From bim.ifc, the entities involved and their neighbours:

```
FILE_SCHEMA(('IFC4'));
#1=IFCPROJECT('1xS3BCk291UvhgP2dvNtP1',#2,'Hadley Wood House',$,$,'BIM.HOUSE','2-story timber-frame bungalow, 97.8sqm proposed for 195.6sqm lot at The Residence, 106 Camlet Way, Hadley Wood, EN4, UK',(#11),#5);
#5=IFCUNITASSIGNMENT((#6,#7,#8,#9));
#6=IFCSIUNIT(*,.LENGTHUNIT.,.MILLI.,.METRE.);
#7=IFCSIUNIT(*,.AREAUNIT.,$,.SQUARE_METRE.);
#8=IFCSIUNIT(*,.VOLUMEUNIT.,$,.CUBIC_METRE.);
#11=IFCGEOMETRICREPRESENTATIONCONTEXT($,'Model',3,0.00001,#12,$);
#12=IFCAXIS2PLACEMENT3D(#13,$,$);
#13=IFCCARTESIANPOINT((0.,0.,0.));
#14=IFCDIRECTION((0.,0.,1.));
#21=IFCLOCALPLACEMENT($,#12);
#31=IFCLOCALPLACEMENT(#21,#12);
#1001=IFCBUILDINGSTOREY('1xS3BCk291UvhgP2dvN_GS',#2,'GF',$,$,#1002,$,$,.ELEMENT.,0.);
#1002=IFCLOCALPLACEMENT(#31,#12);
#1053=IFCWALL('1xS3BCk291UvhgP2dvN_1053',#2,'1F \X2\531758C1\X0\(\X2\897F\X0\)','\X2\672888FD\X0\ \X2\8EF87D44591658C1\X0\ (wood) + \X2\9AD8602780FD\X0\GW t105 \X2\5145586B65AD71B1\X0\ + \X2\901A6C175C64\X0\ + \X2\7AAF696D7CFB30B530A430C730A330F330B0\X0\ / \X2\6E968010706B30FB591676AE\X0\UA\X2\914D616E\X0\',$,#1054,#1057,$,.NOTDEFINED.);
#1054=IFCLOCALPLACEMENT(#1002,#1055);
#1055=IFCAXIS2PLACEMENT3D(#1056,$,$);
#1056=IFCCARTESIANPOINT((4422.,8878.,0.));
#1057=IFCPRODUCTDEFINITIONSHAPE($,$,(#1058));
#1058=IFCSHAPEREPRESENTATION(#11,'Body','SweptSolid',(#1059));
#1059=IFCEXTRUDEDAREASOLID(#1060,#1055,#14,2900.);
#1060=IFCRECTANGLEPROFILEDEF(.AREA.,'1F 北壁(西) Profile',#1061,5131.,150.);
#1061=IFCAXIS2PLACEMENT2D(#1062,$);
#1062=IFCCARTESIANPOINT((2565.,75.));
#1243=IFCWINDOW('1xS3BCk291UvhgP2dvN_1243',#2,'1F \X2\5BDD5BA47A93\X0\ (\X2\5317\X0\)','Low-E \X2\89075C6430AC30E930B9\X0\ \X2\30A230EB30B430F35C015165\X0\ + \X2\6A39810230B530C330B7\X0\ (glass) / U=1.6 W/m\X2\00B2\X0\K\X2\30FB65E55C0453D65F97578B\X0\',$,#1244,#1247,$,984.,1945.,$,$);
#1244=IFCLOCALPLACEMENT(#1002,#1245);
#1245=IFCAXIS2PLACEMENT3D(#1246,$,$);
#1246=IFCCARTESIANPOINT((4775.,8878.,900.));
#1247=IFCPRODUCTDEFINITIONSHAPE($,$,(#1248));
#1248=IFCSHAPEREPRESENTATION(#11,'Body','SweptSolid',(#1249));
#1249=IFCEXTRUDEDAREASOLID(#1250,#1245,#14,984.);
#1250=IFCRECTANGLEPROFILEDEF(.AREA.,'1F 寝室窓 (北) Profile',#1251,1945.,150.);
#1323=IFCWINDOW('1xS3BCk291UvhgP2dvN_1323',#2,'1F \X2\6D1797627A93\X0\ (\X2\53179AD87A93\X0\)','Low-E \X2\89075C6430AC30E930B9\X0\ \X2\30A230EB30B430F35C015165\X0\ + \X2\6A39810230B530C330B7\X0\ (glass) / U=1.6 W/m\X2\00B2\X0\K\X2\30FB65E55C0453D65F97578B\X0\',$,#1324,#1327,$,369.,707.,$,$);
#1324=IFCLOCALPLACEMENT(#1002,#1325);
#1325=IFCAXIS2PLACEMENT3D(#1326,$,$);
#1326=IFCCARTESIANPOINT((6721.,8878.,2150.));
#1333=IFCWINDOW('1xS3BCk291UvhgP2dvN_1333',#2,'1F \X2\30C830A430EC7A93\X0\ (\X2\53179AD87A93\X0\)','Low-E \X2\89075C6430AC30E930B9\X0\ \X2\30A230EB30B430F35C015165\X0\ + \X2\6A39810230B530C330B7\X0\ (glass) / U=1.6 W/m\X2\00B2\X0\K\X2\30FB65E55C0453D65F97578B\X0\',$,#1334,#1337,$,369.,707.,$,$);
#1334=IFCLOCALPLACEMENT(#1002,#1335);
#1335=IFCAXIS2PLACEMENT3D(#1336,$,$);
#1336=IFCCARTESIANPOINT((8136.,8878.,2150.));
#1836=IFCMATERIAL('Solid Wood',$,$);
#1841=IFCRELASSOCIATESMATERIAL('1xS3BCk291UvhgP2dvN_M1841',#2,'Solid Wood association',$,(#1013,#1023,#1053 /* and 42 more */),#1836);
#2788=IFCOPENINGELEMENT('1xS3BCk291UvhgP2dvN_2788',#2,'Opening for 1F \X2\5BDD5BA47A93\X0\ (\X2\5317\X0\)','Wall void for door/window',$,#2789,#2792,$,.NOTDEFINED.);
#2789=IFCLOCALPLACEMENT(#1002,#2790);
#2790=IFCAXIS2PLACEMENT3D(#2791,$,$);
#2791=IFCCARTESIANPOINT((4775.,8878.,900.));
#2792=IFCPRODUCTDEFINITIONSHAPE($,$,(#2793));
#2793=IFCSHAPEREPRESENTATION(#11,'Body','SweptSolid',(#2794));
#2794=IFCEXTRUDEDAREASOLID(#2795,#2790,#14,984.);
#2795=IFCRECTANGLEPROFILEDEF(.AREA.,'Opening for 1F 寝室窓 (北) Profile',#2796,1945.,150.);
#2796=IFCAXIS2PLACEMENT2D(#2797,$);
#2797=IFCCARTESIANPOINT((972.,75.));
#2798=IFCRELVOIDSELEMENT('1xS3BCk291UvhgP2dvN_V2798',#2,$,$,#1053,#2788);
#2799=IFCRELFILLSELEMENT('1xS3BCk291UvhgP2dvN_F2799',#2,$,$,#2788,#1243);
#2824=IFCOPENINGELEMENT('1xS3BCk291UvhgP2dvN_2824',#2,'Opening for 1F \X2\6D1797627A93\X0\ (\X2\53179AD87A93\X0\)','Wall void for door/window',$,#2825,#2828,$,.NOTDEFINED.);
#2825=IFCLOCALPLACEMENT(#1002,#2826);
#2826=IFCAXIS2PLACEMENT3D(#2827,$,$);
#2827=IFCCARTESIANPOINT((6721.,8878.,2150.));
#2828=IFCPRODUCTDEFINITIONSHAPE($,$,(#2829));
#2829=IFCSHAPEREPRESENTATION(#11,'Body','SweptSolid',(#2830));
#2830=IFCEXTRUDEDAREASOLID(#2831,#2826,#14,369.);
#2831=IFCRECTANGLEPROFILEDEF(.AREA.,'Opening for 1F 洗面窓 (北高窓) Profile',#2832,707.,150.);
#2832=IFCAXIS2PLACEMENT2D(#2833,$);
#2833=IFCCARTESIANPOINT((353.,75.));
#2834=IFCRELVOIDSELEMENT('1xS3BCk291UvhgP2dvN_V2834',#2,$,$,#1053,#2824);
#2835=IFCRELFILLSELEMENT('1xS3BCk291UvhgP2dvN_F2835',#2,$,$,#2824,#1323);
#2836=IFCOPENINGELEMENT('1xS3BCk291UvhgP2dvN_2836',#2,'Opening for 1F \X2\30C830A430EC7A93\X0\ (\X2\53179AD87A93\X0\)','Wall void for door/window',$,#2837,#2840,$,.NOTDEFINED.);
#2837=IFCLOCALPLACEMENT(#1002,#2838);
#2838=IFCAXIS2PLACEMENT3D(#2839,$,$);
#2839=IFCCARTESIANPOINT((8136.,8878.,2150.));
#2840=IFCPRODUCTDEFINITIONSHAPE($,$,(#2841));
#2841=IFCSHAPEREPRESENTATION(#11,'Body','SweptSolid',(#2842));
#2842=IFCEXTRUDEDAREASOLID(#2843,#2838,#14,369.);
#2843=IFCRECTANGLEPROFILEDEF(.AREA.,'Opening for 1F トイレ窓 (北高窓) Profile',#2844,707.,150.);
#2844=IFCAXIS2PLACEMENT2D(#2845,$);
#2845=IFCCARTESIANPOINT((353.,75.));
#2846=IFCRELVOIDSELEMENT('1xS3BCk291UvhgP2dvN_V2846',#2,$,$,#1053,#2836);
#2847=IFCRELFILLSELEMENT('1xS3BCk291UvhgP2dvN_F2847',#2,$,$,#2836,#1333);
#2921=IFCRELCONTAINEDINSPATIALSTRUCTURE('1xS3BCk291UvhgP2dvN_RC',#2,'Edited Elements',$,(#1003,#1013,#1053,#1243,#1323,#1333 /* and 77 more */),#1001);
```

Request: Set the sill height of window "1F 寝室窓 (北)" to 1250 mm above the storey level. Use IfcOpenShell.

```python
import numpy as np
import ifcopenshell
import ifcopenshell.api.geometry
import ifcopenshell.geom
import ifcopenshell.util.element
import ifcopenshell.util.placement
import ifcopenshell.util.shape
import ifcopenshell.util.unit

model = ifcopenshell.open("bim.ifc")
unit_scale = ifcopenshell.util.unit.calculate_unit_scale(model)

window = model.by_id(1243)
opening = window.FillsVoids[0].RelatingOpeningElement
storey = ifcopenshell.util.element.get_container(window, ifc_class="IfcBuildingStorey")
level = ifcopenshell.util.placement.get_local_placement(storey.ObjectPlacement)[2, 3]

# The opening's origin need not be at the sill, so measure its lowest point.
shape = ifcopenshell.geom.create_shape(ifcopenshell.geom.settings(), opening)
bottom = ifcopenshell.util.shape.get_shape_bottom_elevation(shape, shape.geometry) / unit_scale
dz = level + 1.25 / unit_scale - bottom

shift = np.array([0.0, 0.0, dz])
# The window is not placed relative to its opening, so move both.
for product in (opening, window):
    matrix = ifcopenshell.util.placement.get_local_placement(product.ObjectPlacement)
    matrix[:3, 3] += shift
    ifcopenshell.api.geometry.edit_object_placement(model, product=product, matrix=matrix, is_si=False)

print(f"moved by {dz * unit_scale:+.3f} m")

model.write("bim-out.ifc")
```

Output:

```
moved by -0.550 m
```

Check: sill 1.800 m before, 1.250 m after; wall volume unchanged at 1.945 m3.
